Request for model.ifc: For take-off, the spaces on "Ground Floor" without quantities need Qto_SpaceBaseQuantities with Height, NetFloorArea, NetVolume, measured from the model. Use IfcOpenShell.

First a look at what the model holds.

```python
import ifcopenshell
import ifcopenshell.util.element
import ifcopenshell.util.unit

model = ifcopenshell.open("model.ifc")
print(model.schema)
for unit_type in ("LENGTHUNIT", "AREAUNIT", "VOLUMEUNIT"):
    print(unit_type, ifcopenshell.util.unit.calculate_unit_scale(model, unit_type))
storey = next(s for s in model.by_type("IfcBuildingStorey") if s.Name == "Ground Floor")
spaces = [e for e in ifcopenshell.util.element.get_decomposition(storey) if e.is_a("IfcSpace")]
for e in sorted(spaces, key=lambda e: e.id()):
    print(e.id(), e.is_a(), e.Name, list(ifcopenshell.util.element.get_psets(e, qtos_only=True)), sep=" | ")
```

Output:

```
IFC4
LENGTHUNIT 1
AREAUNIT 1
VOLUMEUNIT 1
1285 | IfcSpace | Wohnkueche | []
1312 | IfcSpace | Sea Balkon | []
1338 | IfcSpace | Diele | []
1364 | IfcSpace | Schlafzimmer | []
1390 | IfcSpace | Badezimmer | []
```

```python
import ifcopenshell
import ifcopenshell.api.pset
import ifcopenshell.geom
import ifcopenshell.util.element
import ifcopenshell.util.shape
import ifcopenshell.util.unit

model = ifcopenshell.open("model.ifc")
unit_scale = ifcopenshell.util.unit.calculate_unit_scale(model)
area_scale = ifcopenshell.util.unit.calculate_unit_scale(model, "AREAUNIT")
volume_scale = ifcopenshell.util.unit.calculate_unit_scale(model, "VOLUMEUNIT")
settings = ifcopenshell.geom.settings()

storey = next(s for s in model.by_type("IfcBuildingStorey") if s.Name == "Ground Floor")
spaces = [e for e in ifcopenshell.util.element.get_decomposition(storey) if e.is_a("IfcSpace")]

for e in sorted(spaces, key=lambda e: e.id()):
    if ifcopenshell.util.element.get_psets(e, qtos_only=True, should_inherit=False):
        continue
    # Geometry comes back in metres, in the element's own axes.
    shape = ifcopenshell.geom.create_shape(settings, e)
    values = {
        "Height": ifcopenshell.util.shape.get_z(shape.geometry) / unit_scale,
        "NetFloorArea": ifcopenshell.util.shape.get_footprint_area(shape.geometry) / area_scale,
        "NetVolume": ifcopenshell.util.shape.get_volume(shape.geometry) / volume_scale,
    }
    qto = ifcopenshell.api.pset.add_qto(model, product=e, name="Qto_SpaceBaseQuantities")
    ifcopenshell.api.pset.edit_qto(model, qto=qto, properties=values)
    print(e.id(), {k: round(v, 3) for k, v in values.items()})

model.write("model_rev.ifc")
```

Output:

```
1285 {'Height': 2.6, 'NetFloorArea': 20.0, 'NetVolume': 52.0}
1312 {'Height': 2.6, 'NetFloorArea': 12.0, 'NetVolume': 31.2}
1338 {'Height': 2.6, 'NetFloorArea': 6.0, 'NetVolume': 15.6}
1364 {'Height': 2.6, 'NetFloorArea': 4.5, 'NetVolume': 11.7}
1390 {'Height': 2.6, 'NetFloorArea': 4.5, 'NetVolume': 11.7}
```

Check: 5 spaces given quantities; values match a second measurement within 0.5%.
